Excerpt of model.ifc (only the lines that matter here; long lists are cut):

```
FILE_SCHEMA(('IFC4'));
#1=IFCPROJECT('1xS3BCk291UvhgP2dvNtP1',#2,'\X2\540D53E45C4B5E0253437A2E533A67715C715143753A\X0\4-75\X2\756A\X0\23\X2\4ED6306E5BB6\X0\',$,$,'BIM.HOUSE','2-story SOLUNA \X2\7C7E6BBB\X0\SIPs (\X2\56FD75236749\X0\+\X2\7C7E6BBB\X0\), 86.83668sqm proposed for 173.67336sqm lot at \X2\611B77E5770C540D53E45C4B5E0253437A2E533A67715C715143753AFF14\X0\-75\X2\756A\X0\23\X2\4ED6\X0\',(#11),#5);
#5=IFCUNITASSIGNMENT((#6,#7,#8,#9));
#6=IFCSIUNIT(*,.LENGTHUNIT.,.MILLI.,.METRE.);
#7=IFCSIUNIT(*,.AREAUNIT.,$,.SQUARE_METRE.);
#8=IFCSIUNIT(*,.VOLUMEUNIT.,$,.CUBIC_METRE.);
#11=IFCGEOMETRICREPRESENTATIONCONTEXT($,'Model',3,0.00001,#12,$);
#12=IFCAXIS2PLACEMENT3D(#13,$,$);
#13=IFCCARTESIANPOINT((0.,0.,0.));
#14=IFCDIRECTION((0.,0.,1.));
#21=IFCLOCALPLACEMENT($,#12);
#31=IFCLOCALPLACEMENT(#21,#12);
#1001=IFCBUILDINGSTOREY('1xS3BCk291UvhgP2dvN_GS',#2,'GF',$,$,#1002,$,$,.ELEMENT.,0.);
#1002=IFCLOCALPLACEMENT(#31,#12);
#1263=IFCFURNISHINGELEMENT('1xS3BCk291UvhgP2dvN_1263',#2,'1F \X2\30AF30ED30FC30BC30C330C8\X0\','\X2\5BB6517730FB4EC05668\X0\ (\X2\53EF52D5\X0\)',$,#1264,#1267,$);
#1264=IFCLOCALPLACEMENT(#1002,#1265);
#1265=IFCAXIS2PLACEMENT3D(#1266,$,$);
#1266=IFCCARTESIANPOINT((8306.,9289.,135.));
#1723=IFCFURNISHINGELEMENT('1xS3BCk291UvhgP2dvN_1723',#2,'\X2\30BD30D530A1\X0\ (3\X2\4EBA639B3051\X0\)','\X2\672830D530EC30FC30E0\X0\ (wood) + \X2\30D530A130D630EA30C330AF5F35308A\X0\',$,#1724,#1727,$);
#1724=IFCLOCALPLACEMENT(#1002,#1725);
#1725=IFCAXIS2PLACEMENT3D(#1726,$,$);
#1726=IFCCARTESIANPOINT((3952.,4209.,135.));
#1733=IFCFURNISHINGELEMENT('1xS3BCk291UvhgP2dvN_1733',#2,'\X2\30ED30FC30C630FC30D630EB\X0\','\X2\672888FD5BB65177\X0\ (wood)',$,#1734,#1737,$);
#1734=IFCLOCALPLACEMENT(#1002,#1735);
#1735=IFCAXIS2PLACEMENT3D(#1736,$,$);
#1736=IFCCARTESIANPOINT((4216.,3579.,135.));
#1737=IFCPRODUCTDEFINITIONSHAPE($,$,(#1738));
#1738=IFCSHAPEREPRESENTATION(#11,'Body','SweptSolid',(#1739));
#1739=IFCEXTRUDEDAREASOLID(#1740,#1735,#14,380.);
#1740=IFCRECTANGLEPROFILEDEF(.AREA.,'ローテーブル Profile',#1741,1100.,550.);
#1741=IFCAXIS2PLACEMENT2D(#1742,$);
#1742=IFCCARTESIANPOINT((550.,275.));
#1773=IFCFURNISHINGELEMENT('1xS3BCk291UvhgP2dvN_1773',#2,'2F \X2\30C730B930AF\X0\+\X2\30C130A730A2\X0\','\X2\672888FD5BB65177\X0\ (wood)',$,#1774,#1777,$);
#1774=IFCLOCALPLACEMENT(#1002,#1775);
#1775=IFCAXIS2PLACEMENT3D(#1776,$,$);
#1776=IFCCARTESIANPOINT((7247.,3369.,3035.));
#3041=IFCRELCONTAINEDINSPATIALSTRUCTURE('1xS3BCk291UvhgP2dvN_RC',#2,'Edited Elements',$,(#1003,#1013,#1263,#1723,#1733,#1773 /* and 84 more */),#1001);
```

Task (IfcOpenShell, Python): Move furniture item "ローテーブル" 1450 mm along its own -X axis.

```python
import ifcopenshell
import ifcopenshell.api.geometry
import ifcopenshell.util.placement
import ifcopenshell.util.unit

model = ifcopenshell.open("model.ifc")
unit_scale = ifcopenshell.util.unit.calculate_unit_scale(model)

item = model.by_id(1733)
matrix = ifcopenshell.util.placement.get_local_placement(item.ObjectPlacement)
matrix[:3, 3] -= matrix[:3, 0] * 1.45 / unit_scale
ifcopenshell.api.geometry.edit_object_placement(model, product=item, matrix=matrix, is_si=False)

print(ifcopenshell.util.placement.get_local_placement(item.ObjectPlacement).round(3) + 0.0)

model.write("model-out.ifc")
```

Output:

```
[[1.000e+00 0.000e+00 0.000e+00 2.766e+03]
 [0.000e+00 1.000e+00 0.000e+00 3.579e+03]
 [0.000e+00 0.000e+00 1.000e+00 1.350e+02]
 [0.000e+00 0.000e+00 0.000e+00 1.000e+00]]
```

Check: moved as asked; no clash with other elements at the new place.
